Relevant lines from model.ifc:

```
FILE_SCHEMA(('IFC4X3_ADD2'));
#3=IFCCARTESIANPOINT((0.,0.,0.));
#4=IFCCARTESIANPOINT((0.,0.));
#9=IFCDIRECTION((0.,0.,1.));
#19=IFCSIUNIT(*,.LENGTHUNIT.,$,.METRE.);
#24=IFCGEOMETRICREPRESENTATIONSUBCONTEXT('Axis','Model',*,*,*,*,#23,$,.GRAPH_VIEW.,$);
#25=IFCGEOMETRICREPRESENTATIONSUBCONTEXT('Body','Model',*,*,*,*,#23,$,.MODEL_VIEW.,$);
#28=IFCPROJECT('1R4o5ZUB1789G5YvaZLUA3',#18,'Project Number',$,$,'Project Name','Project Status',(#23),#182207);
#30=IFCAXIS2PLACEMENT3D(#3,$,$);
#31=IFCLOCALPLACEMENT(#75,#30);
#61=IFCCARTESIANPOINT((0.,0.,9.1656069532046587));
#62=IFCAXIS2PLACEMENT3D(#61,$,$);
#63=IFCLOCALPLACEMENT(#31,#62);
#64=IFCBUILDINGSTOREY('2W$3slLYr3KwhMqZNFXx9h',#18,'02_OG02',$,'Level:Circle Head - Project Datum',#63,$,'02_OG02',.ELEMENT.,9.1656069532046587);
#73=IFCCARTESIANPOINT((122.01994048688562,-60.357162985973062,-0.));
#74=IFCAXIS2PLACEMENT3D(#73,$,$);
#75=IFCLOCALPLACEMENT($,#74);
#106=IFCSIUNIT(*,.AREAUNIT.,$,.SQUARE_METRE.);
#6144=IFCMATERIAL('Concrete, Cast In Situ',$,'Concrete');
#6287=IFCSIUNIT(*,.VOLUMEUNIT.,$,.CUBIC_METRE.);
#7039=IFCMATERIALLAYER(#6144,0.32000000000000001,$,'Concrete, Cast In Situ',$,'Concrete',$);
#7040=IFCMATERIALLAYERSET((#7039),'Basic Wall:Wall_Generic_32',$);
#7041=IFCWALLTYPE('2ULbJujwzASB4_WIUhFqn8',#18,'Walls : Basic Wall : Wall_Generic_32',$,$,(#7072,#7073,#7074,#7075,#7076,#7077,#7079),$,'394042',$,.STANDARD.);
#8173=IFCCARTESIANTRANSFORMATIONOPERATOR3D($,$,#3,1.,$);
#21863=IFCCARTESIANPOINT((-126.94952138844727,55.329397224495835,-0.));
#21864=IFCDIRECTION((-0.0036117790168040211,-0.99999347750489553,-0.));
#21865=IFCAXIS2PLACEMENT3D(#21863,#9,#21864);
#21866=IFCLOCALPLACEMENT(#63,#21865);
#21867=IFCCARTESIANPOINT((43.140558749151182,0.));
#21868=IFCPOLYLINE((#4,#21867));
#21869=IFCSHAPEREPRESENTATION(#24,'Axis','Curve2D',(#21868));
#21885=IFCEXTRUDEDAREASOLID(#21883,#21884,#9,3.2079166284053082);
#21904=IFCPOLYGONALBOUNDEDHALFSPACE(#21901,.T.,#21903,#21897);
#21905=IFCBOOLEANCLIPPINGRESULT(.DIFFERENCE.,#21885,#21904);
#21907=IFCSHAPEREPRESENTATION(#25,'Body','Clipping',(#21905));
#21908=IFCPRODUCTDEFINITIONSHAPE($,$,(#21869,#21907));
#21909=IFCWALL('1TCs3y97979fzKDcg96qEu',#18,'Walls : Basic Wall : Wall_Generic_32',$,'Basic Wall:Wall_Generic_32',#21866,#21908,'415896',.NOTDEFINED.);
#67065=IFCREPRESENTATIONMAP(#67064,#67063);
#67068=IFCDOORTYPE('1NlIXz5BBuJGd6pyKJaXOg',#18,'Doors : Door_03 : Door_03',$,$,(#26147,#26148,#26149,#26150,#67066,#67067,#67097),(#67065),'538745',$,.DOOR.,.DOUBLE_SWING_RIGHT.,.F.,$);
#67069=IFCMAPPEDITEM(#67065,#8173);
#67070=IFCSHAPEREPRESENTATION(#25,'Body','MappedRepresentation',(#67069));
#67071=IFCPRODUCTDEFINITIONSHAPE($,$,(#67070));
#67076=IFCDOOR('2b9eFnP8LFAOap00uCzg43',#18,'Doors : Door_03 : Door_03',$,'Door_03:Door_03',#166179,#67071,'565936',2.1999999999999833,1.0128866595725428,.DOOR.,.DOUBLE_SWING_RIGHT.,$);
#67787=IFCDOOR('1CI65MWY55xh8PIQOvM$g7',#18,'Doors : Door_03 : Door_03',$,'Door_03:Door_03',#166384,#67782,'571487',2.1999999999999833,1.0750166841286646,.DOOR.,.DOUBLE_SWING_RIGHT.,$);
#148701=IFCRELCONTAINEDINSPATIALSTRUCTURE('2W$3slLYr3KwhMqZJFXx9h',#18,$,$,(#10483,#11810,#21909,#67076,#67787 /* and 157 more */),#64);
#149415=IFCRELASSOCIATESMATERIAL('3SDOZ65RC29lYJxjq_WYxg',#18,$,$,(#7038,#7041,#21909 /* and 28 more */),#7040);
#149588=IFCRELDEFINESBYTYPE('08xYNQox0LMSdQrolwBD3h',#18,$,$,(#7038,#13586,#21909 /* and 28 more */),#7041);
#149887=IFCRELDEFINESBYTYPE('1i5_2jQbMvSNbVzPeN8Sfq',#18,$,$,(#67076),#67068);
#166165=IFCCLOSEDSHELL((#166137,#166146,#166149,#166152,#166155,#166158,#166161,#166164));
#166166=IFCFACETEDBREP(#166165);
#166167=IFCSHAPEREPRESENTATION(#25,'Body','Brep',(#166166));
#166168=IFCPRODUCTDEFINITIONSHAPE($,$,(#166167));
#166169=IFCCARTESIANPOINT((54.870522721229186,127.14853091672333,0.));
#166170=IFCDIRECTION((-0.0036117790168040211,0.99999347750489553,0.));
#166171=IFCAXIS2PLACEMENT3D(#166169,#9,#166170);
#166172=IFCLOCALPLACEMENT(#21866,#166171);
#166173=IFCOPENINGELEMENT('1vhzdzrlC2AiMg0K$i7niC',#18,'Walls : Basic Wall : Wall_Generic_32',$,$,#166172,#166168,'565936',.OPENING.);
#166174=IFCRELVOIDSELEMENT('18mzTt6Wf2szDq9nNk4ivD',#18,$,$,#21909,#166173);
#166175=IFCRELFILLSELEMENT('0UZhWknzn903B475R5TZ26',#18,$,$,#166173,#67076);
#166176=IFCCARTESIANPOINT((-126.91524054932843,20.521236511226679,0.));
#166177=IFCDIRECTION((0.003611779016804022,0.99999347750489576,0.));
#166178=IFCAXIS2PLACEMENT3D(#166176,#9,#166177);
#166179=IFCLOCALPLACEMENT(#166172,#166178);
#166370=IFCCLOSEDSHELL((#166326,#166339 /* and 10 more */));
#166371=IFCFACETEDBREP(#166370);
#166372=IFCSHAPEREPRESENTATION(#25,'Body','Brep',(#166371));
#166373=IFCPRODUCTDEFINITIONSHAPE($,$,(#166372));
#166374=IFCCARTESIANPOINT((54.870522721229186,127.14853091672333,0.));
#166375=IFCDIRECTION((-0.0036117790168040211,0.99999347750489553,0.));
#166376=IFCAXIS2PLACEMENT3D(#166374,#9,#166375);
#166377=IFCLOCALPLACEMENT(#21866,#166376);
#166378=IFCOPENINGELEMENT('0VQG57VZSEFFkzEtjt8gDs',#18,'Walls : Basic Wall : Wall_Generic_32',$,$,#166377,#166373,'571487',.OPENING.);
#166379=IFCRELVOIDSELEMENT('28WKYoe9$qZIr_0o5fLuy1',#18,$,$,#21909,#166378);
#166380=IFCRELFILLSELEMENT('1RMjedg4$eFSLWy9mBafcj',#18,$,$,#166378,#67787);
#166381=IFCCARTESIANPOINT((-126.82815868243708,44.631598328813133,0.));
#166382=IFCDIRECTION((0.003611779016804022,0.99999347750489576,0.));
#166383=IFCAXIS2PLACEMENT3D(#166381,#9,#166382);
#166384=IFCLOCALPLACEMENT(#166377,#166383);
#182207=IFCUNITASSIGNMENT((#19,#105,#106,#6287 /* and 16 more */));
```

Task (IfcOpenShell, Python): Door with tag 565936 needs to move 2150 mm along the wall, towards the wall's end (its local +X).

```python
import ifcopenshell
import ifcopenshell.api.geometry
import ifcopenshell.util.placement

model = ifcopenshell.open("model.ifc")

door = model.by_id(67076)
opening = door.FillsVoids[0].RelatingOpeningElement
wall = opening.VoidsElements[0].RelatingBuildingElement

wall_matrix = ifcopenshell.util.placement.get_local_placement(wall.ObjectPlacement)
shift = wall_matrix[:3, 0] * 2.15
before = ifcopenshell.util.placement.get_local_placement(door.ObjectPlacement)[:3, 3].copy()

# The door is placed relative to its opening, so it follows when the opening moves.
matrix = ifcopenshell.util.placement.get_local_placement(opening.ObjectPlacement)
matrix[:3, 3] += shift
ifcopenshell.api.geometry.edit_object_placement(
    model, product=opening, matrix=matrix, is_si=False, should_transform_children=True
)

after = ifcopenshell.util.placement.get_local_placement(door.ObjectPlacement)[:3, 3]
print("door moved by", (after - before).round(3) + 0.0)

model.write("model_edited.ifc")
```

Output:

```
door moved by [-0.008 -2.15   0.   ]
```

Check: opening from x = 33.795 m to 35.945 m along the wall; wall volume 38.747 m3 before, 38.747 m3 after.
